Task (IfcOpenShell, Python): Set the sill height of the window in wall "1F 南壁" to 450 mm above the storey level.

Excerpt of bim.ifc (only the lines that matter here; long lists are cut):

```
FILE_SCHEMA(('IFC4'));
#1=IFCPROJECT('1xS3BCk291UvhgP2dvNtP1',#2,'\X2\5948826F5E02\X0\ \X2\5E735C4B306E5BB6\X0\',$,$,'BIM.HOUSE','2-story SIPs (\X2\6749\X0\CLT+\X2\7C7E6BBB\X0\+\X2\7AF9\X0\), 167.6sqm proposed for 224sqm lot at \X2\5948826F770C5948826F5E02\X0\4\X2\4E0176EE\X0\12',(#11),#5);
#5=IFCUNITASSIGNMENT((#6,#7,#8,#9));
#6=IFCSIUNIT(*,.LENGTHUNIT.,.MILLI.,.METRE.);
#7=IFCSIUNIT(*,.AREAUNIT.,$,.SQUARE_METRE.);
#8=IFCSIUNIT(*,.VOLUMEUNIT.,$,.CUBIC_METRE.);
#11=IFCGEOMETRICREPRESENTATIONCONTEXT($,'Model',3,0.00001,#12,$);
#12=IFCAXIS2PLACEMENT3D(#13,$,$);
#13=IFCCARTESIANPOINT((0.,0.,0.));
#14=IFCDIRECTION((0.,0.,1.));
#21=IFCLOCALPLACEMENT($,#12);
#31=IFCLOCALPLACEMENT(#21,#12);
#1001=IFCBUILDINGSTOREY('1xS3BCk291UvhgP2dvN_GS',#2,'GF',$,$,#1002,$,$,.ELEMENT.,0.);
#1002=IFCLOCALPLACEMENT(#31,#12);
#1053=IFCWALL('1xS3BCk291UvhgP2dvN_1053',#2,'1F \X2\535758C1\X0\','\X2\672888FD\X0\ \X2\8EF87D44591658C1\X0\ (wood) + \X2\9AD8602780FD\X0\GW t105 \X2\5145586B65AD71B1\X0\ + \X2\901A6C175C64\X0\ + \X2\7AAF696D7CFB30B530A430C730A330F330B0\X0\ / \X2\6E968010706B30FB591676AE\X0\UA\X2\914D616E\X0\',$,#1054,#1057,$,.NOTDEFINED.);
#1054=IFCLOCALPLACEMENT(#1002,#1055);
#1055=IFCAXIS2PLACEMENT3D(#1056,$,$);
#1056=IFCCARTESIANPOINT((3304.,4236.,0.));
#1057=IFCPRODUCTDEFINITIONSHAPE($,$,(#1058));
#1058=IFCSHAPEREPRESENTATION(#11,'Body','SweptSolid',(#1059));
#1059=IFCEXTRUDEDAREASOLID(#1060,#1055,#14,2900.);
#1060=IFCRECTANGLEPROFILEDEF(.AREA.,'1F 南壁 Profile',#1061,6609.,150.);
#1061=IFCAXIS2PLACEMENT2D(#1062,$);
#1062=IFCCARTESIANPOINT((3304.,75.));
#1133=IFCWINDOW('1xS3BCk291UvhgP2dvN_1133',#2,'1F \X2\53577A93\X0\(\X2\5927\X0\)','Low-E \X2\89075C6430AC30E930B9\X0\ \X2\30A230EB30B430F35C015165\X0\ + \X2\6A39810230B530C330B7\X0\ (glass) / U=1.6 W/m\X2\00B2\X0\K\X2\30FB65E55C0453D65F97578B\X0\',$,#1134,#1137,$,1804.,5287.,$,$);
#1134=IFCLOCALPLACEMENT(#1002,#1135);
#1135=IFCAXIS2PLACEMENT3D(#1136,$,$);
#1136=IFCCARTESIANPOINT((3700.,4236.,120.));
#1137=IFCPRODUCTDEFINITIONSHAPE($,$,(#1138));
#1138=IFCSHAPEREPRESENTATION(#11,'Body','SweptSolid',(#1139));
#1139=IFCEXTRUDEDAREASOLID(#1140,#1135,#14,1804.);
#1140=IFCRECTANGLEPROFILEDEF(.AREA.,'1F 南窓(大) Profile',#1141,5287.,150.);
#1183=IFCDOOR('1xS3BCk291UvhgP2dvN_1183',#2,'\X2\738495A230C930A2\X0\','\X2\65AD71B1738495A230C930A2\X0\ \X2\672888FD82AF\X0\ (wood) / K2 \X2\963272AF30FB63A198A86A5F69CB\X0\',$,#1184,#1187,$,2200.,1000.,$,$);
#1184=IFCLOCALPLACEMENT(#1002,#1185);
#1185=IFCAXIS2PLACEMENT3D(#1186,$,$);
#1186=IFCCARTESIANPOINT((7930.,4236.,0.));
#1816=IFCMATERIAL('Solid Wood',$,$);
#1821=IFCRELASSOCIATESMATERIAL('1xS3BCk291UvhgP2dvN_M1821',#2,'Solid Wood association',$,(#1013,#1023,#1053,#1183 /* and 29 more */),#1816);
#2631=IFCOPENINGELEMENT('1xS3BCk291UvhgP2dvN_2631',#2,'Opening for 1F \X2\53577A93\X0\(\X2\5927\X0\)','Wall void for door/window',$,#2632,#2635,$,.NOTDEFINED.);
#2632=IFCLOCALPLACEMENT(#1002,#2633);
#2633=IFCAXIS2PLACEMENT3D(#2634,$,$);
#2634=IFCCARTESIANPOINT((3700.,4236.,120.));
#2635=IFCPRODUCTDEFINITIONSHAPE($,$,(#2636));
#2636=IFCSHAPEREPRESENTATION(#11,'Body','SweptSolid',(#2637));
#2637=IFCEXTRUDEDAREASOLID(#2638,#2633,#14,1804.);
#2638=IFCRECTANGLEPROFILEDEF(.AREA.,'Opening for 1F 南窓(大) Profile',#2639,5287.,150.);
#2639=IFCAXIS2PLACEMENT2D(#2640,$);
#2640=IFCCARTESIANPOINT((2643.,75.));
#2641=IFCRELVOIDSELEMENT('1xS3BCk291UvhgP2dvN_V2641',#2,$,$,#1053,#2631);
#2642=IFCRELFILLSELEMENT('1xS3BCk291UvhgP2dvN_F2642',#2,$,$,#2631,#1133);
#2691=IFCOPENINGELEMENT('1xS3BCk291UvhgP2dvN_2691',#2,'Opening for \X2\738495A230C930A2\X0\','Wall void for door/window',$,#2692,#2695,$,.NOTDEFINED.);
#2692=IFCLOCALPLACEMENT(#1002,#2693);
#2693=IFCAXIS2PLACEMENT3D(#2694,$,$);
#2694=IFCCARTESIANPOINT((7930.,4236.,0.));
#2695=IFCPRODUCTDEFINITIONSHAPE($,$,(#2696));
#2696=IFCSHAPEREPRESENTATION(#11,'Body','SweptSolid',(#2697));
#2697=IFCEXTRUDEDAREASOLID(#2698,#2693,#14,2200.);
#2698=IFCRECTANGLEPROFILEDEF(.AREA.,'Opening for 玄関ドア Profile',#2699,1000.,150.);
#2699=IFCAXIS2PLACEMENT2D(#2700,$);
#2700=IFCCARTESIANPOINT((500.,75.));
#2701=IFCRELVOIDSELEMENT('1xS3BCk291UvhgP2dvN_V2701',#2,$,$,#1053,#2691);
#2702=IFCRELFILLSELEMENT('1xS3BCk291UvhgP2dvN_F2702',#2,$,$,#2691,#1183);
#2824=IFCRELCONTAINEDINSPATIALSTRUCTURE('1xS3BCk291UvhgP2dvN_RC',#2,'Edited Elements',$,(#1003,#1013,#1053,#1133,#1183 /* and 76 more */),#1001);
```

```python
import numpy as np
import ifcopenshell
import ifcopenshell.api.geometry
import ifcopenshell.geom
import ifcopenshell.util.element
import ifcopenshell.util.placement
import ifcopenshell.util.shape
import ifcopenshell.util.unit

model = ifcopenshell.open("bim.ifc")
unit_scale = ifcopenshell.util.unit.calculate_unit_scale(model)

window = model.by_id(1133)
opening = window.FillsVoids[0].RelatingOpeningElement
storey = ifcopenshell.util.element.get_container(window, ifc_class="IfcBuildingStorey")
level = ifcopenshell.util.placement.get_local_placement(storey.ObjectPlacement)[2, 3]

# The opening's origin need not be at the sill, so measure its lowest point.
shape = ifcopenshell.geom.create_shape(ifcopenshell.geom.settings(), opening)
bottom = ifcopenshell.util.shape.get_shape_bottom_elevation(shape, shape.geometry) / unit_scale
dz = level + 0.45 / unit_scale - bottom

shift = np.array([0.0, 0.0, dz])
# The window is not placed relative to its opening, so move both.
for product in (opening, window):
    matrix = ifcopenshell.util.placement.get_local_placement(product.ObjectPlacement)
    matrix[:3, 3] += shift
    ifcopenshell.api.geometry.edit_object_placement(model, product=product, matrix=matrix, is_si=False)

print(f"moved by {dz * unit_scale:+.3f} m")

model.write("bim_rev.ifc")
```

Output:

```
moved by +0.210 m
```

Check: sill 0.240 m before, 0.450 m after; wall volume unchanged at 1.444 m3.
